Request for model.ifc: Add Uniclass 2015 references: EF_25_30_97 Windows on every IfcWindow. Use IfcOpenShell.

First a look at what the model holds.

```python
import ifcopenshell

model = ifcopenshell.open("model.ifc")
print(model.schema)
print("classifications:", [c.Name for c in model.by_type("IfcClassification")])
for ifc_class in ("IfcDoor", "IfcRoof", "IfcStair", "IfcWall", "IfcWindow"):
    print(ifc_class, len(model.by_type(ifc_class)))
```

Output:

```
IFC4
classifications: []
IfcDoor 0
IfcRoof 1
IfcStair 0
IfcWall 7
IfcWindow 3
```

```python
import ifcopenshell
import ifcopenshell.api.classification

model = ifcopenshell.open("model.ifc")

system = ifcopenshell.api.classification.add_classification(model, classification="Uniclass 2015")

codes = {
    "IfcWindow": ("EF_25_30_97", "Windows"),
}
for ifc_class, (code, name) in codes.items():
    products = model.by_type(ifc_class)
    ifcopenshell.api.classification.add_reference(
        model, products=products, classification=system, identification=code, name=name
    )
    print(code, len(products))

model.write("model-out.ifc")
```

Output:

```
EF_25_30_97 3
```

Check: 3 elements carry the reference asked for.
